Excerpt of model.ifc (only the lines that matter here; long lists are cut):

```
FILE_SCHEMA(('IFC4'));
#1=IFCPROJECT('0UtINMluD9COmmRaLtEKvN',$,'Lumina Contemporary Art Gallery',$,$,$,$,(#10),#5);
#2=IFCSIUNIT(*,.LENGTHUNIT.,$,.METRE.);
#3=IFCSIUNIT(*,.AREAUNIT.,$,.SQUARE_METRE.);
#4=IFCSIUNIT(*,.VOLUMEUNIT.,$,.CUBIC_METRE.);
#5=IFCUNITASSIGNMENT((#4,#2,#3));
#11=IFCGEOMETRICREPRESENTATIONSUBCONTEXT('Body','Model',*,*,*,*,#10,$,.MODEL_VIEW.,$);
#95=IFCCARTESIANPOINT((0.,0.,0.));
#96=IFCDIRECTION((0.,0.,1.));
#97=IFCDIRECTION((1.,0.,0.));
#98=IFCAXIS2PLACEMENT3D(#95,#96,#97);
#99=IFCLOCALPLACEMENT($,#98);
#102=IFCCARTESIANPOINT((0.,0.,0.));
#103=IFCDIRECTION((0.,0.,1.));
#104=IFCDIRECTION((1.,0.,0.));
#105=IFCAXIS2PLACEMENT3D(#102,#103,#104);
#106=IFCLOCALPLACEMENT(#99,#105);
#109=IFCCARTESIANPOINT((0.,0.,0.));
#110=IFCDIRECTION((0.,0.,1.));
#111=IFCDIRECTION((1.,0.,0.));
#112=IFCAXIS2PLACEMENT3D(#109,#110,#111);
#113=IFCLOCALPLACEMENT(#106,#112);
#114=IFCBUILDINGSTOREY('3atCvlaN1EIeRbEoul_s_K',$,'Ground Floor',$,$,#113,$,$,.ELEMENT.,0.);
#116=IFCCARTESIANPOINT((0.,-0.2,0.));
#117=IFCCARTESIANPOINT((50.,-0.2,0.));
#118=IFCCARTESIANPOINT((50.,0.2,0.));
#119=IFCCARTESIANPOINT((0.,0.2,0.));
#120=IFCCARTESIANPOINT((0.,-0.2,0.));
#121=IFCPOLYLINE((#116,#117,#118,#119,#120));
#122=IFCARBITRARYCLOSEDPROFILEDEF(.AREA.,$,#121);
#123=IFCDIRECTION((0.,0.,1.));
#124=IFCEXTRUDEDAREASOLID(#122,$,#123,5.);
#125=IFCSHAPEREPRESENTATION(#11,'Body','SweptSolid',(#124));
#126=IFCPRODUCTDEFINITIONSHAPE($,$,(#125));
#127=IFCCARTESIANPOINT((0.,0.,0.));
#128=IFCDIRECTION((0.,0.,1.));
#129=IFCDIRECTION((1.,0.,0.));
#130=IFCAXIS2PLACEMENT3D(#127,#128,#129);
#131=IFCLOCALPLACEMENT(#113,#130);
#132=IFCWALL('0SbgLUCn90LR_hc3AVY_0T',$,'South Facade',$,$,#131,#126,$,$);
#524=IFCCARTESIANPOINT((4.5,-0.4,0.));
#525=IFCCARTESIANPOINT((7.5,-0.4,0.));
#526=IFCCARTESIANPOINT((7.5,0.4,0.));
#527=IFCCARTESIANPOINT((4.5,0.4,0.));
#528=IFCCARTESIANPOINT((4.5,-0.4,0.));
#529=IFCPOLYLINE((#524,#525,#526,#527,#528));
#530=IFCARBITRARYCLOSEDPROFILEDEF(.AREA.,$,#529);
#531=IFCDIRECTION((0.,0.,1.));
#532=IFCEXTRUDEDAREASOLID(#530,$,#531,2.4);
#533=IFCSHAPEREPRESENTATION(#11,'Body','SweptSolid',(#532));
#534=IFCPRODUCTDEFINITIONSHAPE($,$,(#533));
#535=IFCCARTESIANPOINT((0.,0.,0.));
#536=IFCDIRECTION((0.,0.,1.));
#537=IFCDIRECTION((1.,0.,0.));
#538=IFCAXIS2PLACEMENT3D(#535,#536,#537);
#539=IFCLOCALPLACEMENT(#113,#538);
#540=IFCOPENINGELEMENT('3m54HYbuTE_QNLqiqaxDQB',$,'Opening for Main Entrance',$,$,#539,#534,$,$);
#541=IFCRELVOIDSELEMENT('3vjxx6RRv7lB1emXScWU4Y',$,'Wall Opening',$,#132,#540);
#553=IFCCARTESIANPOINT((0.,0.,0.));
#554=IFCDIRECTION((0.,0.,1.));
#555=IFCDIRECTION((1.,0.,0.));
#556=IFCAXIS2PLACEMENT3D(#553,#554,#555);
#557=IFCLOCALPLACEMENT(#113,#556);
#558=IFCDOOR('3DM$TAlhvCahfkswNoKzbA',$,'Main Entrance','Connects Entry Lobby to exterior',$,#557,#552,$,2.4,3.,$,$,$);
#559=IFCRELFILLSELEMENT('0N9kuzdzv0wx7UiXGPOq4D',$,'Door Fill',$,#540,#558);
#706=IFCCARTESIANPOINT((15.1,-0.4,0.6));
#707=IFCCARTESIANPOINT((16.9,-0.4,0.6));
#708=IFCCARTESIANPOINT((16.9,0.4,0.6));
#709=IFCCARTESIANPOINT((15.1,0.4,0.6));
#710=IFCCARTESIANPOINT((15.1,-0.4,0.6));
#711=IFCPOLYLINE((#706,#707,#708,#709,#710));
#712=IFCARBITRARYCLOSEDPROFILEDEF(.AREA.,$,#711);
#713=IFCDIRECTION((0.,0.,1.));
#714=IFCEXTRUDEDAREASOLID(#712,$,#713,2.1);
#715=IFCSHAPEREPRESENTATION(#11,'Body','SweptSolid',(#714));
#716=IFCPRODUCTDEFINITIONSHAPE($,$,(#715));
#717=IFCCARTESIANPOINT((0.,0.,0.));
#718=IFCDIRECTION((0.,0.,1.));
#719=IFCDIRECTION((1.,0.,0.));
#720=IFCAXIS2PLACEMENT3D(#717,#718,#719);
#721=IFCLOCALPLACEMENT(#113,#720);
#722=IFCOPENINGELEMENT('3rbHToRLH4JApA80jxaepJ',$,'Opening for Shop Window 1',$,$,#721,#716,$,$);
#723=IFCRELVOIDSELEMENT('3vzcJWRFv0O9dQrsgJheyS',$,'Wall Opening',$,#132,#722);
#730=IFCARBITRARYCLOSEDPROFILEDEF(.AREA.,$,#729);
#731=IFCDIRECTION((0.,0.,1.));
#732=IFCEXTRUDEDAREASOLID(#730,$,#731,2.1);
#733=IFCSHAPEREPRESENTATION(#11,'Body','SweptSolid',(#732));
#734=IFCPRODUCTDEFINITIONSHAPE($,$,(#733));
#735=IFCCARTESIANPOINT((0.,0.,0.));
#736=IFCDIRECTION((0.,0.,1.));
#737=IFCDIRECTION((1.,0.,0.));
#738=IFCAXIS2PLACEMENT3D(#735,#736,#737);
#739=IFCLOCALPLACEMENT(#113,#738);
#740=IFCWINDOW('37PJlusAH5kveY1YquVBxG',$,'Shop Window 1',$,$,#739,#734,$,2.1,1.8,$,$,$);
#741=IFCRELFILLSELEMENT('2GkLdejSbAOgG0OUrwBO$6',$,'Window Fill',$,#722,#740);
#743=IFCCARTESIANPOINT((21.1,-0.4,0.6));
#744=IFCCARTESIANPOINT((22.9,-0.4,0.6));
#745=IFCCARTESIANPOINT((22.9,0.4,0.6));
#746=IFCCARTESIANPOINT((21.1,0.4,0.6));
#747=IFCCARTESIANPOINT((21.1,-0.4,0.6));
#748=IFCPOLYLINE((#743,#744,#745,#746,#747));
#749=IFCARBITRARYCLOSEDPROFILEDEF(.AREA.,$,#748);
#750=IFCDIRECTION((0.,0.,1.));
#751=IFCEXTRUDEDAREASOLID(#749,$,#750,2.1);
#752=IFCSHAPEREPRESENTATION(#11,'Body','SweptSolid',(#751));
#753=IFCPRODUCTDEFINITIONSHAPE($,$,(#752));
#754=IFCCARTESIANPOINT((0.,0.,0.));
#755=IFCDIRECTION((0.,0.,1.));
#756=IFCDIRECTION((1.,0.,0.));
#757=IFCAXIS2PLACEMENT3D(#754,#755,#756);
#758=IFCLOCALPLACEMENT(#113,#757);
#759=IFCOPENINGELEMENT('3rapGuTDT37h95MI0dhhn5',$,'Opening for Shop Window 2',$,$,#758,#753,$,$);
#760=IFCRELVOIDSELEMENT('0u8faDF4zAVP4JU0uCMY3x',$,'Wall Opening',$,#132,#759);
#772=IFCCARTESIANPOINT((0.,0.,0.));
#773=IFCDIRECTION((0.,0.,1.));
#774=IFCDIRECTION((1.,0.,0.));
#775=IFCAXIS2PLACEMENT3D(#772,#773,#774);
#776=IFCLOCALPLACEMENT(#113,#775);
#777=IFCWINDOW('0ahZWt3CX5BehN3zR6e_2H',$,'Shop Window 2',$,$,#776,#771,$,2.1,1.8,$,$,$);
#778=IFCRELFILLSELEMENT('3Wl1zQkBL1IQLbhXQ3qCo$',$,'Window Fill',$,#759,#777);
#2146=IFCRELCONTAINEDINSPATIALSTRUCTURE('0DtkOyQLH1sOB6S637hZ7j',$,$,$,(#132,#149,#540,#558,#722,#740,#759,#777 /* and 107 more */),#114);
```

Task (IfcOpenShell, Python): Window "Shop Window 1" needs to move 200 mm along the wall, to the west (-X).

```python
import ifcopenshell
import ifcopenshell.api.geometry
import ifcopenshell.util.placement
import ifcopenshell.util.unit

model = ifcopenshell.open("model.ifc")
unit_scale = ifcopenshell.util.unit.calculate_unit_scale(model)

window = model.by_id(740)
opening = window.FillsVoids[0].RelatingOpeningElement
wall = opening.VoidsElements[0].RelatingBuildingElement

wall_matrix = ifcopenshell.util.placement.get_local_placement(wall.ObjectPlacement)
shift = wall_matrix[:3, 0] * -0.2 / unit_scale
before = ifcopenshell.util.placement.get_local_placement(window.ObjectPlacement)[:3, 3].copy()

# The window is not placed relative to its opening, so move both.
for product in (opening, window):
    matrix = ifcopenshell.util.placement.get_local_placement(product.ObjectPlacement)
    matrix[:3, 3] += shift
    ifcopenshell.api.geometry.edit_object_placement(model, product=product, matrix=matrix, is_si=False)

after = ifcopenshell.util.placement.get_local_placement(window.ObjectPlacement)[:3, 3]
print("window moved by", (after - before).round(3) + 0.0)

model.write("model_v2.ifc")
```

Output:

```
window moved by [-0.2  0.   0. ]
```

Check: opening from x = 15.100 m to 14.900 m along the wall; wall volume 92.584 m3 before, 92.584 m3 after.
